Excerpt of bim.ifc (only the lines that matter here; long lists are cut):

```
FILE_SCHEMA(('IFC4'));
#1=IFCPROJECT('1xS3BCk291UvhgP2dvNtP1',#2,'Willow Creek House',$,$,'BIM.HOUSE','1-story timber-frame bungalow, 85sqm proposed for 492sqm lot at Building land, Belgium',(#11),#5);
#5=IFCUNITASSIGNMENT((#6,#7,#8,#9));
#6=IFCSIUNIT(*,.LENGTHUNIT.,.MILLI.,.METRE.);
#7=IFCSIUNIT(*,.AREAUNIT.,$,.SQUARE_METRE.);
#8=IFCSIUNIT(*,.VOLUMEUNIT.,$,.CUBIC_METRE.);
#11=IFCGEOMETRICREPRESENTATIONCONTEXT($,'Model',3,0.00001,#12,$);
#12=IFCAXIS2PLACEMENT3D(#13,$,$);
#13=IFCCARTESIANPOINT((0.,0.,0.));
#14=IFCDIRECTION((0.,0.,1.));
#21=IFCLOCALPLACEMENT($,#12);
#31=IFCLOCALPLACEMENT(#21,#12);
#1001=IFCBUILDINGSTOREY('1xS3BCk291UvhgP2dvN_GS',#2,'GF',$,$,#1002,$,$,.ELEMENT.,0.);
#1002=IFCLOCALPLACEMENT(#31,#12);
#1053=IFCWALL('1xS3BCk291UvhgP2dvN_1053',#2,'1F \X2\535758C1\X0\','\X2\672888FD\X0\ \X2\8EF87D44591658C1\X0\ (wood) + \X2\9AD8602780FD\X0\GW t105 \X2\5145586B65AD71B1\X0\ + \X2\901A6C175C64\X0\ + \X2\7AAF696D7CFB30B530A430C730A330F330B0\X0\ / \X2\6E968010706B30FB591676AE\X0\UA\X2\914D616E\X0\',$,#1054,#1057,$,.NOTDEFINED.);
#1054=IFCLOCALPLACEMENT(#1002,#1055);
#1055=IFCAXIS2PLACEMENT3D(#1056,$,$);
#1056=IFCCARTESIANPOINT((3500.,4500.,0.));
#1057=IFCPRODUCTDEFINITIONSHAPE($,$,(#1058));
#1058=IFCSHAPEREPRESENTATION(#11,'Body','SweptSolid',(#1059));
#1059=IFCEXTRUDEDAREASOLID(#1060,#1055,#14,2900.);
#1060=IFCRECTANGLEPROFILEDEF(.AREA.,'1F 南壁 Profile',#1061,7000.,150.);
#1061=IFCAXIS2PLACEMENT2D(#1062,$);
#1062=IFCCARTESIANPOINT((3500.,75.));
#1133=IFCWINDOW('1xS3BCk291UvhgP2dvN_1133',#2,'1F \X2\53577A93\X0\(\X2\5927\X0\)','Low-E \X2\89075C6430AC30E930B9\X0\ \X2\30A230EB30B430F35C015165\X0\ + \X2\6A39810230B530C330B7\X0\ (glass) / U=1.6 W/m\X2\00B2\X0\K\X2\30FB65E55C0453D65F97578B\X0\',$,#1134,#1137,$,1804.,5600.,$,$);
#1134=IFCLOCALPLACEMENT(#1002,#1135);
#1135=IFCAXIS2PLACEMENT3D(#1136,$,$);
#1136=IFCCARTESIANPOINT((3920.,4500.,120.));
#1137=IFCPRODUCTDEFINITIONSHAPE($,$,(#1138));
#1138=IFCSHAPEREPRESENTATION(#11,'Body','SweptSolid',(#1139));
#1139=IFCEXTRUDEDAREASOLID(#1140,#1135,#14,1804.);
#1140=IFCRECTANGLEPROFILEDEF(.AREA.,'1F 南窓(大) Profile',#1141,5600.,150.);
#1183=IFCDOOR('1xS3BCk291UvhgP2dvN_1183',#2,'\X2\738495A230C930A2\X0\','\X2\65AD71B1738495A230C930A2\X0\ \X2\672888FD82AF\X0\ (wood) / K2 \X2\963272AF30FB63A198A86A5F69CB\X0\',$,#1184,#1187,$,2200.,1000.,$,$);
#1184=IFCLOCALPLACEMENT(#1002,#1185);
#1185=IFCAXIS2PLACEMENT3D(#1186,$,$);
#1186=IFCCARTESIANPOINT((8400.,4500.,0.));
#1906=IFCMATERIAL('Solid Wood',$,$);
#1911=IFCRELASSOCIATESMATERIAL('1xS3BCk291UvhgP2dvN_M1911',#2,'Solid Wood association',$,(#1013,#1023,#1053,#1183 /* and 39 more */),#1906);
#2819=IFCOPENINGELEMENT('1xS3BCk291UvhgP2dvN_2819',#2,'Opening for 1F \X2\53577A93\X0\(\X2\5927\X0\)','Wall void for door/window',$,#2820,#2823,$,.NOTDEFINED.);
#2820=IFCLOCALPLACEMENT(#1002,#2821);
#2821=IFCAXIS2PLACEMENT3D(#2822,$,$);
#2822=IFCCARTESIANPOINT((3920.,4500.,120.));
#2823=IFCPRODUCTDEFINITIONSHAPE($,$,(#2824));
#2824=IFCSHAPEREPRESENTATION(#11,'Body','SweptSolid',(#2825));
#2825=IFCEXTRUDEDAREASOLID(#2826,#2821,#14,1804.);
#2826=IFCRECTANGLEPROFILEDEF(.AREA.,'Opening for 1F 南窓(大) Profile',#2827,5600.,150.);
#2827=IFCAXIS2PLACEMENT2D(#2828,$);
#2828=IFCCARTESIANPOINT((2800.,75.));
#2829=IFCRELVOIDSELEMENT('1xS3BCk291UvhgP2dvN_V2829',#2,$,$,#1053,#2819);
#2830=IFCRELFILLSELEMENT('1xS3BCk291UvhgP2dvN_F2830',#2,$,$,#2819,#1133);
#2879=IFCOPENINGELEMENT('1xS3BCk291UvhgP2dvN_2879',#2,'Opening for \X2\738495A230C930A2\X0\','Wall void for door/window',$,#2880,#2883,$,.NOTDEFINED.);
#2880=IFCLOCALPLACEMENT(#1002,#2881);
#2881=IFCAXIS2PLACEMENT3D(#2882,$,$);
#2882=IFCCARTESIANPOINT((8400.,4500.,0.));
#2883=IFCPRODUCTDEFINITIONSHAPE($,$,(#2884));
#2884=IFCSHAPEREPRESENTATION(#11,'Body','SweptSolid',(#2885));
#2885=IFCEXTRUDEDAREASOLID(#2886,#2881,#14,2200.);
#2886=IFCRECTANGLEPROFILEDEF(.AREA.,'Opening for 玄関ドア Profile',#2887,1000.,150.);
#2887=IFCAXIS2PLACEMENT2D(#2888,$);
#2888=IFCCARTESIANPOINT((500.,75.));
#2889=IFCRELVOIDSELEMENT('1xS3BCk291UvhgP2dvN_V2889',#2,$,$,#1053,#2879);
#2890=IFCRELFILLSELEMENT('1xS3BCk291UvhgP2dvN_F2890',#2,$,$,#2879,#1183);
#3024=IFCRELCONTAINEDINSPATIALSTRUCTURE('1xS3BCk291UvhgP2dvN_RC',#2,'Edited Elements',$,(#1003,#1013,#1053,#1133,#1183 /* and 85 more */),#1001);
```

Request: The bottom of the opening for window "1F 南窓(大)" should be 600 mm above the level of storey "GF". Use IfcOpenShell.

```python
import numpy as np
import ifcopenshell
import ifcopenshell.api.geometry
import ifcopenshell.geom
import ifcopenshell.util.element
import ifcopenshell.util.placement
import ifcopenshell.util.shape
import ifcopenshell.util.unit

model = ifcopenshell.open("bim.ifc")
unit_scale = ifcopenshell.util.unit.calculate_unit_scale(model)

window = model.by_id(1133)
opening = window.FillsVoids[0].RelatingOpeningElement
storey = ifcopenshell.util.element.get_container(window, ifc_class="IfcBuildingStorey")
level = ifcopenshell.util.placement.get_local_placement(storey.ObjectPlacement)[2, 3]

# The opening's origin need not be at the sill, so measure its lowest point.
shape = ifcopenshell.geom.create_shape(ifcopenshell.geom.settings(), opening)
bottom = ifcopenshell.util.shape.get_shape_bottom_elevation(shape, shape.geometry) / unit_scale
dz = level + 600.0 - bottom

shift = np.array([0.0, 0.0, dz])
# The window is not placed relative to its opening, so move both.
for product in (opening, window):
    matrix = ifcopenshell.util.placement.get_local_placement(product.ObjectPlacement)
    matrix[:3, 3] += shift
    ifcopenshell.api.geometry.edit_object_placement(model, product=product, matrix=matrix, is_si=False)

print(f"moved by {dz * unit_scale:+.3f} m")

model.write("bim_v2.ifc")
```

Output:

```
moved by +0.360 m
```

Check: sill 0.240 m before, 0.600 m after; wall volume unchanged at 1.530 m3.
